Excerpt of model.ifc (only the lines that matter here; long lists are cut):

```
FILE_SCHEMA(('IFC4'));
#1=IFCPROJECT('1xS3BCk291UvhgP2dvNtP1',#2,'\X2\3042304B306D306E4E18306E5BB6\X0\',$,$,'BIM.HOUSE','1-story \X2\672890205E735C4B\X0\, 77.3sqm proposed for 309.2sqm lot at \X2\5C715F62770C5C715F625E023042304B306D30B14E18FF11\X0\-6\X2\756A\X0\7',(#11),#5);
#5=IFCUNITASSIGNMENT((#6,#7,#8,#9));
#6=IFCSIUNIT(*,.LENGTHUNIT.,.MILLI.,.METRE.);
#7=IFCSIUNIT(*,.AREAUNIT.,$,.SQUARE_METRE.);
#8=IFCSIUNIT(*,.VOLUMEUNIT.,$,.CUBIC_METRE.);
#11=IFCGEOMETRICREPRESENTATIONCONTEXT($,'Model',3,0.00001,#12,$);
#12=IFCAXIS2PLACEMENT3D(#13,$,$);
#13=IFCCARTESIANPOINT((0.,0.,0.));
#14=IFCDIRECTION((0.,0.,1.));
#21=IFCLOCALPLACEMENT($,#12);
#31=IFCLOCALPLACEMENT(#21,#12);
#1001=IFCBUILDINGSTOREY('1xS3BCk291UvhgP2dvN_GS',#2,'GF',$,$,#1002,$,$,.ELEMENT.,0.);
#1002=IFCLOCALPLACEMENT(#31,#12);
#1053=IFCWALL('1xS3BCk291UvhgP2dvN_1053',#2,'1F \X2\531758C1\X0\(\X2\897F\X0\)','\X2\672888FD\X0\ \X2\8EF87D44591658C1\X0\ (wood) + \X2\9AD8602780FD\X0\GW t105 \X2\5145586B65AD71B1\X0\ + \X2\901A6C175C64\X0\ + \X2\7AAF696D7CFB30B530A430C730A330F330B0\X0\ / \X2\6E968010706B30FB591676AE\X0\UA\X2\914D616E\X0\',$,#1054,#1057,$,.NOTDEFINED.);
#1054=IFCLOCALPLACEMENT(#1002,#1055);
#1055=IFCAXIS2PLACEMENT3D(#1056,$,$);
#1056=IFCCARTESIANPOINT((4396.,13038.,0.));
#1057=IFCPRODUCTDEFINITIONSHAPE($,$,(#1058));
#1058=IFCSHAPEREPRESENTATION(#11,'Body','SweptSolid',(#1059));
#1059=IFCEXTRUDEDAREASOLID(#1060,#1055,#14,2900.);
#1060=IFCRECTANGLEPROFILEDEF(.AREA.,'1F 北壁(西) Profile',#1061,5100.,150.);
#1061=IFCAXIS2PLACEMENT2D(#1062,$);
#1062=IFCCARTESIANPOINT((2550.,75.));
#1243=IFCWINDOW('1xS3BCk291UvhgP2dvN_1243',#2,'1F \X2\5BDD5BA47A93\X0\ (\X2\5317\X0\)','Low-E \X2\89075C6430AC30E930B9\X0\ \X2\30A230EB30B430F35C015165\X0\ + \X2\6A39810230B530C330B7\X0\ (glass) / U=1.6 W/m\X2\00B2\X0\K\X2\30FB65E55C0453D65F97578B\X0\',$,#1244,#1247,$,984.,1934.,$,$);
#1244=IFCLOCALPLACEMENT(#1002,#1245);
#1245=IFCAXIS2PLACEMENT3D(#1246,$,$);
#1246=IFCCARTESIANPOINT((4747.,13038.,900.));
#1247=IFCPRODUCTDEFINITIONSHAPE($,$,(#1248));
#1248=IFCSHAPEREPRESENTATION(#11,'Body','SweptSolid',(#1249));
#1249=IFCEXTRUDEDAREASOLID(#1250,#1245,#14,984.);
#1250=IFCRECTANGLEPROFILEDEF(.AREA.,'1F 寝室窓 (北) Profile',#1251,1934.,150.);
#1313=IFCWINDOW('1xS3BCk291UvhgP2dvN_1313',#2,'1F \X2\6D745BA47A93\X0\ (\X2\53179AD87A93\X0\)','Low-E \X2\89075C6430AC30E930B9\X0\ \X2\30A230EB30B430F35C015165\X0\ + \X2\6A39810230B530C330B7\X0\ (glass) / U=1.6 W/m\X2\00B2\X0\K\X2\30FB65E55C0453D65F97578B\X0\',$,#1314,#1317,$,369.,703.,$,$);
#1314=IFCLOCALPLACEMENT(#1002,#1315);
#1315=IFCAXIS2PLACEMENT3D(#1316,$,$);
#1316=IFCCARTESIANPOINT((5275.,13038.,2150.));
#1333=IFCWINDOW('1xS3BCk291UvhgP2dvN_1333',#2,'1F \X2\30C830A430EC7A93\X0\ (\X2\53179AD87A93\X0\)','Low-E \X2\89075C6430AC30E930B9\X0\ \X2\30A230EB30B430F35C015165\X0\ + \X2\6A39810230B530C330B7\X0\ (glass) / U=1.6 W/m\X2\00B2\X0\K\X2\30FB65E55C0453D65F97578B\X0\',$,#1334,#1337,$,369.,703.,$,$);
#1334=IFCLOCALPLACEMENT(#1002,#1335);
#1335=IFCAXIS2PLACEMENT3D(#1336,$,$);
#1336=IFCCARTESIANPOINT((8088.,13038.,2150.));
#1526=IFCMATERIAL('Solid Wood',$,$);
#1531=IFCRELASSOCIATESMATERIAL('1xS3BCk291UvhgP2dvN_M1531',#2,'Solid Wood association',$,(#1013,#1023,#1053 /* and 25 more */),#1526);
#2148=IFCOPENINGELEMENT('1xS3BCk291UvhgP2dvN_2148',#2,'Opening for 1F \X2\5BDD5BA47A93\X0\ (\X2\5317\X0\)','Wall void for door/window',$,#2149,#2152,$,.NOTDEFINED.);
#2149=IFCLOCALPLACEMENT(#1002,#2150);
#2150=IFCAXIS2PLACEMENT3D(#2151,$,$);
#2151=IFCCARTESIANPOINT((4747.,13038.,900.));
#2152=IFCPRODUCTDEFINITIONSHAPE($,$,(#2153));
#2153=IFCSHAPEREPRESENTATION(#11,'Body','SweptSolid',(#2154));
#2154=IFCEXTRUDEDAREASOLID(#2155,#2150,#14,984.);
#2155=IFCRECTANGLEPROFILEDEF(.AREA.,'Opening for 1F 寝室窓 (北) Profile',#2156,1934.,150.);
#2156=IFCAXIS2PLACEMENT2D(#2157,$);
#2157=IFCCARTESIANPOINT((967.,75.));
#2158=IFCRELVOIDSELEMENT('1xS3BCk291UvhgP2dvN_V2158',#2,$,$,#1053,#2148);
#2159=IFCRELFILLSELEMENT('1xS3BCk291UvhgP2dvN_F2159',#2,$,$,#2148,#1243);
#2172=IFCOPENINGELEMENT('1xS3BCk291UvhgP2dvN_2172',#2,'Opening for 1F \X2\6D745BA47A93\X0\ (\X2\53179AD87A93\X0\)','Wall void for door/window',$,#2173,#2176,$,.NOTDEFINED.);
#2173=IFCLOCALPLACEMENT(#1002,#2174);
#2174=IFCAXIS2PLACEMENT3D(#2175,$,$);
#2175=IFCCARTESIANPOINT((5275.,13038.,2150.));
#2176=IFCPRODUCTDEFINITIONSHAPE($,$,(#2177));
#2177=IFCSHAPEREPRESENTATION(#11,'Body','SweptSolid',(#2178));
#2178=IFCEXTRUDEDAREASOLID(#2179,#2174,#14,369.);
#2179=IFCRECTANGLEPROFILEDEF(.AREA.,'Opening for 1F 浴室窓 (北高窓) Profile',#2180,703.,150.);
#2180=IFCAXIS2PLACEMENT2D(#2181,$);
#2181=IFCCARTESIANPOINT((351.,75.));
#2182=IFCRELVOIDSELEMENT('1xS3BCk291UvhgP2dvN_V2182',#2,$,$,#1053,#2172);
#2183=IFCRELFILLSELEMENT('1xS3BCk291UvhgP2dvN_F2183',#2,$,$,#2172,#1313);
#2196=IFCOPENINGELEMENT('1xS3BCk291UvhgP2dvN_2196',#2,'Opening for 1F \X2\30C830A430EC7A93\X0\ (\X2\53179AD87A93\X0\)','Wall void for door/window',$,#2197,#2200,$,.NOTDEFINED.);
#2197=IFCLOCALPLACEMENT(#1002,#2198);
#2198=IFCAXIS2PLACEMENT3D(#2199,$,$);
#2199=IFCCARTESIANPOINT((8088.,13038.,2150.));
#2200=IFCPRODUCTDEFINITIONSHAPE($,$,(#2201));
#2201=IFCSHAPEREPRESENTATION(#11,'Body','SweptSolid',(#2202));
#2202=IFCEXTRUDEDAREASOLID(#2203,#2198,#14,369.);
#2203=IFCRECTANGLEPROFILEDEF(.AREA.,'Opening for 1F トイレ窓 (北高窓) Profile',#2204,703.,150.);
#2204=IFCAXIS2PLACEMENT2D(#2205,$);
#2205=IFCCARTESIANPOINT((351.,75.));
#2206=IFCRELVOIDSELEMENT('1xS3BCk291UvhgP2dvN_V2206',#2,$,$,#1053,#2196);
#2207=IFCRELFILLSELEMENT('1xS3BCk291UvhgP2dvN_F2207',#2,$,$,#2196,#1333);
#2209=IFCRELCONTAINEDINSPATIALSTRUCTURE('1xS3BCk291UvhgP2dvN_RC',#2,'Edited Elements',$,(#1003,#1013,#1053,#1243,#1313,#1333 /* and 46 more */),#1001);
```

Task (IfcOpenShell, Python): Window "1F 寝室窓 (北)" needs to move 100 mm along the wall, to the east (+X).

```python
import ifcopenshell
import ifcopenshell.api.geometry
import ifcopenshell.util.placement

model = ifcopenshell.open("model.ifc")

window = model.by_guid("1xS3BCk291UvhgP2dvN_1243")
opening = window.FillsVoids[0].RelatingOpeningElement
wall = opening.VoidsElements[0].RelatingBuildingElement

wall_matrix = ifcopenshell.util.placement.get_local_placement(wall.ObjectPlacement)
shift = wall_matrix[:3, 0] * 100.0
before = ifcopenshell.util.placement.get_local_placement(window.ObjectPlacement)[:3, 3].copy()

# The window is not placed relative to its opening, so move both.
for product in (opening, window):
    matrix = ifcopenshell.util.placement.get_local_placement(product.ObjectPlacement)
    matrix[:3, 3] += shift
    ifcopenshell.api.geometry.edit_object_placement(model, product=product, matrix=matrix, is_si=False)

after = ifcopenshell.util.placement.get_local_placement(window.ObjectPlacement)[:3, 3]
print("window moved by", (after - before).round(3) + 0.0)

model.write("model_v2.ifc")
```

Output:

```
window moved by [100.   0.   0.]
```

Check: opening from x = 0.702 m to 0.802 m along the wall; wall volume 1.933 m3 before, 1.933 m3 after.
